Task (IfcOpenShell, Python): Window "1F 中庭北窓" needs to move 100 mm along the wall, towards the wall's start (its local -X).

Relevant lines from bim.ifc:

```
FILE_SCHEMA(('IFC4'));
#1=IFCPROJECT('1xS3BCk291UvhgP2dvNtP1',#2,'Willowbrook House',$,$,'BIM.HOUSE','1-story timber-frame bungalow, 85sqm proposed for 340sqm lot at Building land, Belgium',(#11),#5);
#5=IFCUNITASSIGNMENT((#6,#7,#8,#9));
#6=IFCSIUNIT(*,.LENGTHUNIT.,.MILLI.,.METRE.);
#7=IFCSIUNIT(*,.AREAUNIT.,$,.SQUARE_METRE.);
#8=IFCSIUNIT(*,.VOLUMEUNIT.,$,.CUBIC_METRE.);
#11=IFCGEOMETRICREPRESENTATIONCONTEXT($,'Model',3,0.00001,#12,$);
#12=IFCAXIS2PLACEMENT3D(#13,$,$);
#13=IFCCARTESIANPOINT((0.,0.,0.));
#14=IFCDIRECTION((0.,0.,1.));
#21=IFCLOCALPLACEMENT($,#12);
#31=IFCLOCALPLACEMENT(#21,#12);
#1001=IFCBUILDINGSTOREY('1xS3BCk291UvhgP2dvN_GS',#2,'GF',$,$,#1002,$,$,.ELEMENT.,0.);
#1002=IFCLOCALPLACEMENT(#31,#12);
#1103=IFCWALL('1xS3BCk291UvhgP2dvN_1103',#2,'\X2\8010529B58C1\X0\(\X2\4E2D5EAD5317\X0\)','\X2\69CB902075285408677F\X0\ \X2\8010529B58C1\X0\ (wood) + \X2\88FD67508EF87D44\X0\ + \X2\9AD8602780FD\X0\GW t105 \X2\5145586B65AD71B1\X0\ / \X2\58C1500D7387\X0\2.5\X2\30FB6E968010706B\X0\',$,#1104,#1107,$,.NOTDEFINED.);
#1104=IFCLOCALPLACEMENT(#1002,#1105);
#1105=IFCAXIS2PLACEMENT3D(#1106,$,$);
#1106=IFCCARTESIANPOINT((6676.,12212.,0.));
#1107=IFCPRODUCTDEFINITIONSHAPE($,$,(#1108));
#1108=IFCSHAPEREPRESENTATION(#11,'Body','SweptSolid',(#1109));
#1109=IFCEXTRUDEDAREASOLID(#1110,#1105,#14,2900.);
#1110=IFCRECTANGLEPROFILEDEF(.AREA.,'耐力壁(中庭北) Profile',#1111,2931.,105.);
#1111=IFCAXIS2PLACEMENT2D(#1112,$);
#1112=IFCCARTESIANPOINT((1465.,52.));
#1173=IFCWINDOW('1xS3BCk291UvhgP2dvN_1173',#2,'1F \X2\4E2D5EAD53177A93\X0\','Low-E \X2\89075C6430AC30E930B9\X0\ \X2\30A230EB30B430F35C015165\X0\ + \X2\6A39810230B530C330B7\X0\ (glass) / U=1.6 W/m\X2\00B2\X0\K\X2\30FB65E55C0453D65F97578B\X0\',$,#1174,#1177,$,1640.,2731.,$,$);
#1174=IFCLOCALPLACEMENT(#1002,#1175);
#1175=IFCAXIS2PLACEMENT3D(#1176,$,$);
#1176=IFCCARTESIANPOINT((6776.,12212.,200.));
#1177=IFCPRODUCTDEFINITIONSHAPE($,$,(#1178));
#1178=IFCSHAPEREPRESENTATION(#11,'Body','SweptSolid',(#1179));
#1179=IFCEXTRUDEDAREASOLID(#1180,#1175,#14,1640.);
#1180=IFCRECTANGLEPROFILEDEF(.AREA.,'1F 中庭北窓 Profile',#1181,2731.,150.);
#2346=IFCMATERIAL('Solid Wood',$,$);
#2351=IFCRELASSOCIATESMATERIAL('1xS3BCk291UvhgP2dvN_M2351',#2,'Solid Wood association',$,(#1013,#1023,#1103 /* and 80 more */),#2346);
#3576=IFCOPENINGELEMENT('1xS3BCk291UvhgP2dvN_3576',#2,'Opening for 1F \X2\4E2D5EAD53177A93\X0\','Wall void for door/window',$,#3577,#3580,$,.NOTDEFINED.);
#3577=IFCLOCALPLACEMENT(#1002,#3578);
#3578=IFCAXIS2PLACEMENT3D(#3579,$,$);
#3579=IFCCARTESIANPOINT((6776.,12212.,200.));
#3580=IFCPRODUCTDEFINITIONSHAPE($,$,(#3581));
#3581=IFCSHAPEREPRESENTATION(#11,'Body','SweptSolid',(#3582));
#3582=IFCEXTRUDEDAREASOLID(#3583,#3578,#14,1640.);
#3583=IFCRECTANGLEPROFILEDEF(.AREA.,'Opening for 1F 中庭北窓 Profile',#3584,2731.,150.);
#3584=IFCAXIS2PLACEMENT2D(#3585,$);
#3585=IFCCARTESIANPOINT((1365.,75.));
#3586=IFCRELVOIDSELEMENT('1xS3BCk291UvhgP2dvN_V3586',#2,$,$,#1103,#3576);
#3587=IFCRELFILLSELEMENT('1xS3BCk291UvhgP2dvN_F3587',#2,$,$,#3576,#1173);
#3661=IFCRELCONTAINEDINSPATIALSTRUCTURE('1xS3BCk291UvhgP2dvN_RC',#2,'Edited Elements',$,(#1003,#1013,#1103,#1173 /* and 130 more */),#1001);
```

```python
import ifcopenshell
import ifcopenshell.api.geometry
import ifcopenshell.util.placement
import ifcopenshell.util.unit

model = ifcopenshell.open("bim.ifc")
unit_scale = ifcopenshell.util.unit.calculate_unit_scale(model)

window = model.by_guid("1xS3BCk291UvhgP2dvN_1173")
opening = window.FillsVoids[0].RelatingOpeningElement
wall = opening.VoidsElements[0].RelatingBuildingElement

wall_matrix = ifcopenshell.util.placement.get_local_placement(wall.ObjectPlacement)
shift = wall_matrix[:3, 0] * -0.1 / unit_scale
before = ifcopenshell.util.placement.get_local_placement(window.ObjectPlacement)[:3, 3].copy()

# The window is not placed relative to its opening, so move both.
for product in (opening, window):
    matrix = ifcopenshell.util.placement.get_local_placement(product.ObjectPlacement)
    matrix[:3, 3] += shift
    ifcopenshell.api.geometry.edit_object_placement(model, product=product, matrix=matrix, is_si=False)

after = ifcopenshell.util.placement.get_local_placement(window.ObjectPlacement)[:3, 3]
print("window moved by", (after - before).round(3) + 0.0)

model.write("bim_v2.ifc")
```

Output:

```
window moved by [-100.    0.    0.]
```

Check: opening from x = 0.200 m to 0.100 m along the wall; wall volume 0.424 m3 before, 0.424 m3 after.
